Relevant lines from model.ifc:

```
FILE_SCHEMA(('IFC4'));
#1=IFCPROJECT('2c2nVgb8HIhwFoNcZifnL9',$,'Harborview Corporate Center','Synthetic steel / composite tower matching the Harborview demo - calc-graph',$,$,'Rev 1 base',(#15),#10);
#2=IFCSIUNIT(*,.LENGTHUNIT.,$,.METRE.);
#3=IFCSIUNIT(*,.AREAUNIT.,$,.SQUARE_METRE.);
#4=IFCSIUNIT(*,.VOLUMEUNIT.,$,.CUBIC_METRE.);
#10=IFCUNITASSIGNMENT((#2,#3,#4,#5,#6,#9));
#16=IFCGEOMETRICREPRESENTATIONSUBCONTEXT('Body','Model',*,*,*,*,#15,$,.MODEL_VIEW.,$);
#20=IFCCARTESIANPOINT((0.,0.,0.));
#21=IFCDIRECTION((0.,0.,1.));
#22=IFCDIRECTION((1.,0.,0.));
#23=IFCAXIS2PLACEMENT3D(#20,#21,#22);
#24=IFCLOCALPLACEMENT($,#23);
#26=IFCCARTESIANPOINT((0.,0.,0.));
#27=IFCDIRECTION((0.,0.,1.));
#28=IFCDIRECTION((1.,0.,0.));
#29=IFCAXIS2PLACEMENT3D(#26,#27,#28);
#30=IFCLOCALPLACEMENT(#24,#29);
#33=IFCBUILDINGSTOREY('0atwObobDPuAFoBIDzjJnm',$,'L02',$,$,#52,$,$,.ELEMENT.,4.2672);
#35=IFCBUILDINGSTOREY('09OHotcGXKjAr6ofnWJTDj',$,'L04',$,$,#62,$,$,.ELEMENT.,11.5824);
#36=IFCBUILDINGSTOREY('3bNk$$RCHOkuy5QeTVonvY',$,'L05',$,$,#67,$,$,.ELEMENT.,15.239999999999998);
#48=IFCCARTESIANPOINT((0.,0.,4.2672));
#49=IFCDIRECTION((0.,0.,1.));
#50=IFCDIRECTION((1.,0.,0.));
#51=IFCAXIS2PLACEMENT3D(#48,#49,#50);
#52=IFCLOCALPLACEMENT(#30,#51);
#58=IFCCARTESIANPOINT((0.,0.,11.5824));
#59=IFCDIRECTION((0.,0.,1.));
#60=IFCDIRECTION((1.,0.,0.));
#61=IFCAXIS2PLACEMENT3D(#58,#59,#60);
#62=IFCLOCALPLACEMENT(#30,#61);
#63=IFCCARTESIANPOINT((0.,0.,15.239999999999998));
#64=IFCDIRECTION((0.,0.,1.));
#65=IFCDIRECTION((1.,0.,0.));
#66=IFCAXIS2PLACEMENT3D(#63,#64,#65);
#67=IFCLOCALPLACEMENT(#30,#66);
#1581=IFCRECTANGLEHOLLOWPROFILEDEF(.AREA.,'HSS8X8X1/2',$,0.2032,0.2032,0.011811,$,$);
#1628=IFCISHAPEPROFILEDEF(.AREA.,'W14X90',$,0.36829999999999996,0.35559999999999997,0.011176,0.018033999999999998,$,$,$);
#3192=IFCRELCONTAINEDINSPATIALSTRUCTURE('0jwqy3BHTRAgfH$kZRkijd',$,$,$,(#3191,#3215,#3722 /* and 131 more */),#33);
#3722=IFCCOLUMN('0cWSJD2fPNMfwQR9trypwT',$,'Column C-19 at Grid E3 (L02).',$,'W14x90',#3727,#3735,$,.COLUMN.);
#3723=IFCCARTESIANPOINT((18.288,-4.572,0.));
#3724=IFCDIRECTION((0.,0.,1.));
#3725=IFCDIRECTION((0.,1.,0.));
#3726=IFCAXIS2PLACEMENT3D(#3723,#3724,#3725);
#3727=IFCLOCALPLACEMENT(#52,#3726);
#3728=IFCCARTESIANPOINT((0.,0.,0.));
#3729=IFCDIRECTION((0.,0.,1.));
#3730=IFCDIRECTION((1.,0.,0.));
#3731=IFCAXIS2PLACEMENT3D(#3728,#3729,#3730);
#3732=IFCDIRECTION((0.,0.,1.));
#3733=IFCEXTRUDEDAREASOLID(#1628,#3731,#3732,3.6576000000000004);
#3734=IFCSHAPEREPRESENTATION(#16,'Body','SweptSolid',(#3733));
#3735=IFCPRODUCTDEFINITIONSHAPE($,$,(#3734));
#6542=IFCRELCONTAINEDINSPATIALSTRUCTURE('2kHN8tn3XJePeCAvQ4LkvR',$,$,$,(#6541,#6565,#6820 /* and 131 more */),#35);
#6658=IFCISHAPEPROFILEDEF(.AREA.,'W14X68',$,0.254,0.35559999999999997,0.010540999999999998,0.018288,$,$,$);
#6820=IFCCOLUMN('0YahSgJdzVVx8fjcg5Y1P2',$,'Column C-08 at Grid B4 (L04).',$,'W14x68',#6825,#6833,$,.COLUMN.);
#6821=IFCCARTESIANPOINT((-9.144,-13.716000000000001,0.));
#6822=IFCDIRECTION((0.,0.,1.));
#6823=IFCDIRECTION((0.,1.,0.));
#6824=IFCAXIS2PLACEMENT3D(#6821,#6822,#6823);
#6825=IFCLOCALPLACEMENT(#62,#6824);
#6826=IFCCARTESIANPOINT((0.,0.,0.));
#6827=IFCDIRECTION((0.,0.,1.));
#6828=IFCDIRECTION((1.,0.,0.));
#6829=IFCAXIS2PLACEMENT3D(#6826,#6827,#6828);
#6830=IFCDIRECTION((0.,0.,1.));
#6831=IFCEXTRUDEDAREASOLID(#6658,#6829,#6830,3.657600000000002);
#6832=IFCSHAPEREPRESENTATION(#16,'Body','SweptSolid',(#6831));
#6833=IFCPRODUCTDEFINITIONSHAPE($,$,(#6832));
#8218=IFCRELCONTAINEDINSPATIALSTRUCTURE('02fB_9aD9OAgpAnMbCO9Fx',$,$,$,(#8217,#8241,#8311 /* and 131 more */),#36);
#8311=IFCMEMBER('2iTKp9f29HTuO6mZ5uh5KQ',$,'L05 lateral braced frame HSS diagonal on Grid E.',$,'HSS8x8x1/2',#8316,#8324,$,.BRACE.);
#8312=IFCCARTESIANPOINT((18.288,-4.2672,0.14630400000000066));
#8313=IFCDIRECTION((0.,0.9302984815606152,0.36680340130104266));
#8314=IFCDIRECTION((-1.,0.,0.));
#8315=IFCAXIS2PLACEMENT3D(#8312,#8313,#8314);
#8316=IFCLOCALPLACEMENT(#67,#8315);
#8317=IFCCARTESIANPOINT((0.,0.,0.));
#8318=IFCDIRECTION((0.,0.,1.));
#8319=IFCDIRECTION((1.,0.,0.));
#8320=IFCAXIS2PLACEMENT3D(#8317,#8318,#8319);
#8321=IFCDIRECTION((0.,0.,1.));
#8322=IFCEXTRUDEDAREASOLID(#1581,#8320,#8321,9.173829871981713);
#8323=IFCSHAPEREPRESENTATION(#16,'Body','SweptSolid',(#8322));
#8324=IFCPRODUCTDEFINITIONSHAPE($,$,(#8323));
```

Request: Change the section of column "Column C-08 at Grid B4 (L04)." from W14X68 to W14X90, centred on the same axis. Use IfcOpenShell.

```python
import ifcopenshell
import ifcopenshell.util.element
import ifcopenshell.util.representation

model = ifcopenshell.open("model.ifc")

member = model.by_id(6820)
source = next(p for p in model.by_type("IfcIShapeProfileDef") if p.ProfileName == "W14X90")

body = ifcopenshell.util.representation.get_representation(member, "Model", "Body")
solid = body.Items[0]
old_profile = solid.SweptArea

# Copy the section's sizes but keep this member's own profile position.
profile = ifcopenshell.util.element.copy(model, source)
profile.Position = old_profile.Position
solid.SweptArea = profile
if not model.get_total_inverses(old_profile):
    ifcopenshell.util.element.remove_deep2(model, old_profile)

print(solid.SweptArea)

model.write("model_edited.ifc")
```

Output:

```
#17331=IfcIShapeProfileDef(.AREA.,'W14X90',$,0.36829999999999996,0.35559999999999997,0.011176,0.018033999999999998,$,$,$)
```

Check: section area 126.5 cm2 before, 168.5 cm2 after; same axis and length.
